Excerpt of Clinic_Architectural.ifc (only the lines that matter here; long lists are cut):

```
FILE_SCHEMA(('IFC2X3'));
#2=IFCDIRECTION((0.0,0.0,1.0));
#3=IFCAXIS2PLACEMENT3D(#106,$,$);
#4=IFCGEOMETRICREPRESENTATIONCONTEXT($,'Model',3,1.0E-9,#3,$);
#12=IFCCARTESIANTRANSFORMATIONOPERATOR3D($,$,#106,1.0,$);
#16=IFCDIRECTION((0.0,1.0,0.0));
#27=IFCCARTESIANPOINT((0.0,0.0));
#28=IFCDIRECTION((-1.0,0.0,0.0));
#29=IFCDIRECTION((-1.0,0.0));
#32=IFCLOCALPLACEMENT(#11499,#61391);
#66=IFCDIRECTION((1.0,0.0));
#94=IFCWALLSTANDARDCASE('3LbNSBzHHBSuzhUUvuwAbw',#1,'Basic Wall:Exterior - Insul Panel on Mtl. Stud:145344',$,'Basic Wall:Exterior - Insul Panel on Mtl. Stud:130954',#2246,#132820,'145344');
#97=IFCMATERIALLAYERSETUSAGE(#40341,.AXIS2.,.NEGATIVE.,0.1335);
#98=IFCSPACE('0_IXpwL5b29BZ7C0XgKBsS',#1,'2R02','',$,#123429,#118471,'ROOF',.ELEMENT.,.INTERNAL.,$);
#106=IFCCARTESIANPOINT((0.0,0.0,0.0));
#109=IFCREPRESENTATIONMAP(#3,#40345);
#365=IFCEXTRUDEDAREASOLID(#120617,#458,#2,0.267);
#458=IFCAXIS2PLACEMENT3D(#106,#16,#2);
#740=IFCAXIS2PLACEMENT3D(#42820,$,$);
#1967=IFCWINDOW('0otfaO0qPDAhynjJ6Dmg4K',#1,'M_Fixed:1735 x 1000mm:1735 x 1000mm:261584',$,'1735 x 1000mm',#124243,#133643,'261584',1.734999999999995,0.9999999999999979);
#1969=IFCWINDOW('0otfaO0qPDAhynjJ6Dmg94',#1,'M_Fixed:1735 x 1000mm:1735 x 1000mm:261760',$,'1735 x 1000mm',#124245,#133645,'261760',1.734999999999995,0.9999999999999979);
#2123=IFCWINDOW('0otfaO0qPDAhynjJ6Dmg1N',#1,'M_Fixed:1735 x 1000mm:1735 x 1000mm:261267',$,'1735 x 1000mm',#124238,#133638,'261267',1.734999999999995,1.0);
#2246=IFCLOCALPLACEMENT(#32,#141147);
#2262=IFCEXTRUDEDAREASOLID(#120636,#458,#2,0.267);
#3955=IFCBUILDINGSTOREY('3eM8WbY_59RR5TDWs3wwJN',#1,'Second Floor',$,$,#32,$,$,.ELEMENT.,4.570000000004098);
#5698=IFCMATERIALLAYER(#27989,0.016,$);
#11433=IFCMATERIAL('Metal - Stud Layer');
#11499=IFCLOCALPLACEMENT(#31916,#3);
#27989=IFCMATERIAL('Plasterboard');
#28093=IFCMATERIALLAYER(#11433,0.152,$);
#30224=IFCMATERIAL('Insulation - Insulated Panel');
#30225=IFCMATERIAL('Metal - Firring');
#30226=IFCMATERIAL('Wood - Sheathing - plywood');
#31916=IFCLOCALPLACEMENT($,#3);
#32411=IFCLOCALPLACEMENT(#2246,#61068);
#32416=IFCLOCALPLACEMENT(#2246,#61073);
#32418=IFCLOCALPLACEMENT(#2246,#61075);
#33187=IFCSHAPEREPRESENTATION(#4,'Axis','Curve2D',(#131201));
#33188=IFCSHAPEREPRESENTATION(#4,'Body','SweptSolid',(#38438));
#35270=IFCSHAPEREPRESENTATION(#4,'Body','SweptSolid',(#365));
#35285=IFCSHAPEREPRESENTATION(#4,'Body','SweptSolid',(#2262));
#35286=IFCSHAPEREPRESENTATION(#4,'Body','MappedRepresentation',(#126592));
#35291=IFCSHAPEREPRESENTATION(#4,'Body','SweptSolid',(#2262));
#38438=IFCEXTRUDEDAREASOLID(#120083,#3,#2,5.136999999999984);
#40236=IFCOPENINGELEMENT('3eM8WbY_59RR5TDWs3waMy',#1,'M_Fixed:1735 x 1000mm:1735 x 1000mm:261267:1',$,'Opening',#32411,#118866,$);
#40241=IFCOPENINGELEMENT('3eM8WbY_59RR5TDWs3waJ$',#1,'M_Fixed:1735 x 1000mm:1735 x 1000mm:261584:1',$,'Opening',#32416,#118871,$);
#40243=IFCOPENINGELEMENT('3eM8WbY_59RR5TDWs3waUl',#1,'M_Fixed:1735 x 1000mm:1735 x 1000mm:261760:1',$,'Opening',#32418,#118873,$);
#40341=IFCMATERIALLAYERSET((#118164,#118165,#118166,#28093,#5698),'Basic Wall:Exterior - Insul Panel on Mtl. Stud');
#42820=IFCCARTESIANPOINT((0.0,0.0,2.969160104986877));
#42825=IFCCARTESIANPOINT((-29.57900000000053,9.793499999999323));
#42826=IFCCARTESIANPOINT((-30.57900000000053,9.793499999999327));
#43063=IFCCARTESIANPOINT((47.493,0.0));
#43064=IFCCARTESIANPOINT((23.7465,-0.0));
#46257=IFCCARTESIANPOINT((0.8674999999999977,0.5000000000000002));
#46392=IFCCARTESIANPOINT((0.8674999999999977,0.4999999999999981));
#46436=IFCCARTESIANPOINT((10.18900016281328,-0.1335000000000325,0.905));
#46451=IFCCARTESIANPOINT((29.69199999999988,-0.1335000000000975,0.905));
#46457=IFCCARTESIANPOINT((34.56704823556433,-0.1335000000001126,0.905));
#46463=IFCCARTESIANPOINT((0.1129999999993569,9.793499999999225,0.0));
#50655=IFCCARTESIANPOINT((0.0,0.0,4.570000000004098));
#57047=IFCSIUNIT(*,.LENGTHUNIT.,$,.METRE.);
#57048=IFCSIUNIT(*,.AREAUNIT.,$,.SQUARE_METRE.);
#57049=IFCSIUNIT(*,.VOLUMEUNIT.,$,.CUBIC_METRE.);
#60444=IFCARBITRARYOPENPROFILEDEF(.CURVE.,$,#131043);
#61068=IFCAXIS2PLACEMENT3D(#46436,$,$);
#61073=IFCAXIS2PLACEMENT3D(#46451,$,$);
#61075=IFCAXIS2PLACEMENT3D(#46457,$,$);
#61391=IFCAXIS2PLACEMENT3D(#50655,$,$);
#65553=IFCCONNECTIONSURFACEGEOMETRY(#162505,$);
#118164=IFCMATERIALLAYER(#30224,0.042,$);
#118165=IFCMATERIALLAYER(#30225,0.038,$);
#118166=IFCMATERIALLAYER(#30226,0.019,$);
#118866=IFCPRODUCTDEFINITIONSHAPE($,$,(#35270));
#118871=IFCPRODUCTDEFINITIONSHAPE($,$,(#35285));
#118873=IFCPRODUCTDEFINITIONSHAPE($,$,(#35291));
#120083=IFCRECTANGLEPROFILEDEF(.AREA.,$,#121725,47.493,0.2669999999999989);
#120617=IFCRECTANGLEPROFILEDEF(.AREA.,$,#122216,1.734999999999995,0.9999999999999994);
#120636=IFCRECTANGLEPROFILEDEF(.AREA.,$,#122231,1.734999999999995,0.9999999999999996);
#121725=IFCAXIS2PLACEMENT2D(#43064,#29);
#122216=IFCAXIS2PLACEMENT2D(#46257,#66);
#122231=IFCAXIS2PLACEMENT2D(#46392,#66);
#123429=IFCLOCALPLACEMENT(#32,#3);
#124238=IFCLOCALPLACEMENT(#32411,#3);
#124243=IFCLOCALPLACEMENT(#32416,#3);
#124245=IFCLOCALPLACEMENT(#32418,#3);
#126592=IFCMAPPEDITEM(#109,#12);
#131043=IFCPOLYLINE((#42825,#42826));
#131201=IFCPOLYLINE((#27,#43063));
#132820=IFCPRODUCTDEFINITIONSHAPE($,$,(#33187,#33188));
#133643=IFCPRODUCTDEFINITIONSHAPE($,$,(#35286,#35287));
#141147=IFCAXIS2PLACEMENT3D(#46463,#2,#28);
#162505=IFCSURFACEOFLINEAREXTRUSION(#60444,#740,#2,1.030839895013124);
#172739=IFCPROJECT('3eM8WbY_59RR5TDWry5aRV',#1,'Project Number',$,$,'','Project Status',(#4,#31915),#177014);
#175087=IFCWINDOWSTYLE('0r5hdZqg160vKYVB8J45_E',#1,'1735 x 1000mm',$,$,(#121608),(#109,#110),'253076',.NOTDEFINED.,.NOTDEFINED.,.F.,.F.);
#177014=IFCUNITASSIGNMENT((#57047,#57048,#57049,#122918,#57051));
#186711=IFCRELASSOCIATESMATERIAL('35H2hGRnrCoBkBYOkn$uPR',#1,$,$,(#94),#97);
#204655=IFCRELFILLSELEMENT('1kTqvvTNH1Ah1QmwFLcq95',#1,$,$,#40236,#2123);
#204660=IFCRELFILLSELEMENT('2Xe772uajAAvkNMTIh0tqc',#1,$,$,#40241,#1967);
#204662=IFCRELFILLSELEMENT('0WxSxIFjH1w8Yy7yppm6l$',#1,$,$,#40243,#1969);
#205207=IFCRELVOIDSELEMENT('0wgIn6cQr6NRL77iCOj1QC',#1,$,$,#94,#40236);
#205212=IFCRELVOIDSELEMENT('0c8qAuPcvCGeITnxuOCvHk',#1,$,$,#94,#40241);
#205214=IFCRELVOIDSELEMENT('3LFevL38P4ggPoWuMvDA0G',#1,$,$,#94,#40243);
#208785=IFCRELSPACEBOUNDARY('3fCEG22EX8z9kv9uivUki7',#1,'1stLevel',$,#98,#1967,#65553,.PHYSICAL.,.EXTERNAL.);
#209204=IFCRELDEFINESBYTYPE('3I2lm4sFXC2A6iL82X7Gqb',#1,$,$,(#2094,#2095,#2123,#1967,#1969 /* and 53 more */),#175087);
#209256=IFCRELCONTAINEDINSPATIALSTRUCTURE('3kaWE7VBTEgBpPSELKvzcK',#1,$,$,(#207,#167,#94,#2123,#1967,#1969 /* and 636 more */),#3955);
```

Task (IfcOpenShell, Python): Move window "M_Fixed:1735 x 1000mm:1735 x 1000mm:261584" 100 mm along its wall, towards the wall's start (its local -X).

```python
import numpy as np
import ifcopenshell
import ifcopenshell.api.geometry
import ifcopenshell.util.placement

model = ifcopenshell.open("Clinic_Architectural.ifc")

window = model.by_guid("0otfaO0qPDAhynjJ6Dmg4K")
opening = window.FillsVoids[0].RelatingOpeningElement
wall = opening.VoidsElements[0].RelatingBuildingElement

wall_matrix = ifcopenshell.util.placement.get_local_placement(wall.ObjectPlacement)
shift = wall_matrix[:3, 0] * -0.1
before = ifcopenshell.util.placement.get_local_placement(window.ObjectPlacement)[:3, 3].copy()

# The window is placed relative to its opening, so it follows when the opening moves.
matrix = ifcopenshell.util.placement.get_local_placement(opening.ObjectPlacement)
matrix[:3, 3] += shift
ifcopenshell.api.geometry.edit_object_placement(
    model, product=opening, matrix=matrix, is_si=False, should_transform_children=True
)

# Space boundary surfaces are stored in each space's coordinates; move them too.
for rel in window.ProvidesBoundaries:
    if not rel.ConnectionGeometry:
        continue
    surface = rel.ConnectionGeometry.SurfaceOnRelatingElement
    space_matrix = ifcopenshell.util.placement.get_local_placement(rel.RelatingSpace.ObjectPlacement)
    point = np.array(surface.Position.Location.Coordinates) + space_matrix[:3, :3].T @ shift
    surface.Position = model.createIfcAxis2Placement3D(
        model.createIfcCartesianPoint(point.tolist()), surface.Position.Axis, surface.Position.RefDirection
    )

after = ifcopenshell.util.placement.get_local_placement(window.ObjectPlacement)[:3, 3]
print("window moved by", (after - before).round(3) + 0.0)

model.write("Clinic_Architectural_edited.ifc")
```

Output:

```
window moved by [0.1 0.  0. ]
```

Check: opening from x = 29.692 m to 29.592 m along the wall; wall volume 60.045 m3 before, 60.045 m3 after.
